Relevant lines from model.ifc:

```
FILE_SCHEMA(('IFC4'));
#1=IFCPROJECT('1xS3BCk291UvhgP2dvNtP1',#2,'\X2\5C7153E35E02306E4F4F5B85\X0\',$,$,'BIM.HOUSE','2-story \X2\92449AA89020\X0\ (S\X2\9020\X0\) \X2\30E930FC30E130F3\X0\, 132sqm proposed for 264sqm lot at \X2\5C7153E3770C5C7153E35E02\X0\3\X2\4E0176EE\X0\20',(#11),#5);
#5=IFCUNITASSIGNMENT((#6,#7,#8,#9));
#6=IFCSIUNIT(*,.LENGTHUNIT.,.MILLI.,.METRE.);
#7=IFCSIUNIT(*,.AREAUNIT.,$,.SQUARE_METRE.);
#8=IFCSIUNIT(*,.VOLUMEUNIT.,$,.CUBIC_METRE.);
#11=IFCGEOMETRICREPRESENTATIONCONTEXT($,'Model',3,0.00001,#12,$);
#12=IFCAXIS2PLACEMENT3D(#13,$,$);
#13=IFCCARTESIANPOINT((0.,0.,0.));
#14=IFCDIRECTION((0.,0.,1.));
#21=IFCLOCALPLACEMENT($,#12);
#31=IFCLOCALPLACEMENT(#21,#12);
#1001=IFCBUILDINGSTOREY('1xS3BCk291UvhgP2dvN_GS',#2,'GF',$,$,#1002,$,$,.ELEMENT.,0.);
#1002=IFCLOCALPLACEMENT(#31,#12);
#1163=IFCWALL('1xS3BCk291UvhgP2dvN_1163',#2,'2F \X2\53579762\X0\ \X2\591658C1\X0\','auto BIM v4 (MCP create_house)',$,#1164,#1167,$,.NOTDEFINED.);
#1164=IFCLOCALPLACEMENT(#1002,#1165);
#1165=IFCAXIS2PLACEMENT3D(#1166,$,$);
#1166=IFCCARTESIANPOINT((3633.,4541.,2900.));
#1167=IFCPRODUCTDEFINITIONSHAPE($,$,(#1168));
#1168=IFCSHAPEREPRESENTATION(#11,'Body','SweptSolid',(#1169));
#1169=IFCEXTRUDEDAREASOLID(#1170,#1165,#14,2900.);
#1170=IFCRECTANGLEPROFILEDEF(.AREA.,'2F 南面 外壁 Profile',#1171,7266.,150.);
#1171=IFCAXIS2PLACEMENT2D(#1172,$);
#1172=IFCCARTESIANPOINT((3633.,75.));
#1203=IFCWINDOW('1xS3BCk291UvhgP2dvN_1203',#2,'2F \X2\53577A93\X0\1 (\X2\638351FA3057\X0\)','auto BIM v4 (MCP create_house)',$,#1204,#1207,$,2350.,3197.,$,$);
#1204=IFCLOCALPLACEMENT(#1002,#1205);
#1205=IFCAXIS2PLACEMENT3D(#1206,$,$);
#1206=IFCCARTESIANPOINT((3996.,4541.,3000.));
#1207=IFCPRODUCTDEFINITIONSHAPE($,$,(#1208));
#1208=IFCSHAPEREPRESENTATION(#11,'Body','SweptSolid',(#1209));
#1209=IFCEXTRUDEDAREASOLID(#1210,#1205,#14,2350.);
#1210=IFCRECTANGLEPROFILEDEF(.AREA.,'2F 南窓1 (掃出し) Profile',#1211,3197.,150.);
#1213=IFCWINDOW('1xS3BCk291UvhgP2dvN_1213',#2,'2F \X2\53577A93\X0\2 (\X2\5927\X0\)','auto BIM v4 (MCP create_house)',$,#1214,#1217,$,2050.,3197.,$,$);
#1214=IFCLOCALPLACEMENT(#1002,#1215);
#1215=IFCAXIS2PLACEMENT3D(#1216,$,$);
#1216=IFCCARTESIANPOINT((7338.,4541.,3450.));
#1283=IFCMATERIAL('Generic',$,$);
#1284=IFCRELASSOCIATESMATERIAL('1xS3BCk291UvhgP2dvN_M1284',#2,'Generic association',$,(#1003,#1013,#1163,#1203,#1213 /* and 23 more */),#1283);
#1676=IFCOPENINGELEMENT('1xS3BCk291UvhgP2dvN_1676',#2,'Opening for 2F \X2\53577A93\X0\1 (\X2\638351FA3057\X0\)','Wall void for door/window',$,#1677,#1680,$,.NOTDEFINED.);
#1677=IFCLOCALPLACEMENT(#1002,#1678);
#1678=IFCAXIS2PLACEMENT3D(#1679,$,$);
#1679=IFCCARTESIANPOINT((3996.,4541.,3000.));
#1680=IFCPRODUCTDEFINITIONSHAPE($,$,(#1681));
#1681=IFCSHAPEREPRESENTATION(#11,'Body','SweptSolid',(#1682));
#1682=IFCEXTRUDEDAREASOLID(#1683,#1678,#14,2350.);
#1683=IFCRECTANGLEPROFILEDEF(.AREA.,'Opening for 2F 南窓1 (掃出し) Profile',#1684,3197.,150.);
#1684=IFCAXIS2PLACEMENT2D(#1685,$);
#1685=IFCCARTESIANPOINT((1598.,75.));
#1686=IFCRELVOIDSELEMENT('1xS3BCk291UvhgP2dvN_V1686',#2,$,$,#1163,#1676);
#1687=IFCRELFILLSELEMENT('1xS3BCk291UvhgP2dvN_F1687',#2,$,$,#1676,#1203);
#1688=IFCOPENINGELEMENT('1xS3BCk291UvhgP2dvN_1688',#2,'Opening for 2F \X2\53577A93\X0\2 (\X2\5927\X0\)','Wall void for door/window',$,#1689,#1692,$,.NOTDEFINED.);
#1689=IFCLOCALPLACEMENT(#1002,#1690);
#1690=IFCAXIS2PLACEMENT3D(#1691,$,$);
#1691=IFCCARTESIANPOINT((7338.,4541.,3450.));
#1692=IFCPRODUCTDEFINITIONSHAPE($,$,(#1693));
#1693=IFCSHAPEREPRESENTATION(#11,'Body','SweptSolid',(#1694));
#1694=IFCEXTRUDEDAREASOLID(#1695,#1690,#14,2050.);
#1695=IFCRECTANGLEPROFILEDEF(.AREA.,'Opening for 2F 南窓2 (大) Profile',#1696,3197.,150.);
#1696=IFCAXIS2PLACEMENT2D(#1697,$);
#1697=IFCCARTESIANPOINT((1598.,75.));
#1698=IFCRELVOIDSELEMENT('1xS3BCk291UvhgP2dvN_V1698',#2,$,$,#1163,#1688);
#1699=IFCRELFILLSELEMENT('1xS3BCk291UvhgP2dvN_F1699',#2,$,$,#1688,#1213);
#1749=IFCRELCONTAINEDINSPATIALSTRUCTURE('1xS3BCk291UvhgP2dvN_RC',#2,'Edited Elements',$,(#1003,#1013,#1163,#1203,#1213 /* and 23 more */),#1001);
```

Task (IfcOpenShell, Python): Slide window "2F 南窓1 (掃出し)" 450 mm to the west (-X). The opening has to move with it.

```python
import ifcopenshell
import ifcopenshell.api.geometry
import ifcopenshell.util.placement

model = ifcopenshell.open("model.ifc")

window = model.by_id(1203)
opening = window.FillsVoids[0].RelatingOpeningElement
wall = opening.VoidsElements[0].RelatingBuildingElement

wall_matrix = ifcopenshell.util.placement.get_local_placement(wall.ObjectPlacement)
shift = wall_matrix[:3, 0] * -450.0
before = ifcopenshell.util.placement.get_local_placement(window.ObjectPlacement)[:3, 3].copy()

# The window is not placed relative to its opening, so move both.
for product in (opening, window):
    matrix = ifcopenshell.util.placement.get_local_placement(product.ObjectPlacement)
    matrix[:3, 3] += shift
    ifcopenshell.api.geometry.edit_object_placement(model, product=product, matrix=matrix, is_si=False)

after = ifcopenshell.util.placement.get_local_placement(window.ObjectPlacement)[:3, 3]
print("window moved by", (after - before).round(3) + 0.0)

model.write("model_v2.ifc")
```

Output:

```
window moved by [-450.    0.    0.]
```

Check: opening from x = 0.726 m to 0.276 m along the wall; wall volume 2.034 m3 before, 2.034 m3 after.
